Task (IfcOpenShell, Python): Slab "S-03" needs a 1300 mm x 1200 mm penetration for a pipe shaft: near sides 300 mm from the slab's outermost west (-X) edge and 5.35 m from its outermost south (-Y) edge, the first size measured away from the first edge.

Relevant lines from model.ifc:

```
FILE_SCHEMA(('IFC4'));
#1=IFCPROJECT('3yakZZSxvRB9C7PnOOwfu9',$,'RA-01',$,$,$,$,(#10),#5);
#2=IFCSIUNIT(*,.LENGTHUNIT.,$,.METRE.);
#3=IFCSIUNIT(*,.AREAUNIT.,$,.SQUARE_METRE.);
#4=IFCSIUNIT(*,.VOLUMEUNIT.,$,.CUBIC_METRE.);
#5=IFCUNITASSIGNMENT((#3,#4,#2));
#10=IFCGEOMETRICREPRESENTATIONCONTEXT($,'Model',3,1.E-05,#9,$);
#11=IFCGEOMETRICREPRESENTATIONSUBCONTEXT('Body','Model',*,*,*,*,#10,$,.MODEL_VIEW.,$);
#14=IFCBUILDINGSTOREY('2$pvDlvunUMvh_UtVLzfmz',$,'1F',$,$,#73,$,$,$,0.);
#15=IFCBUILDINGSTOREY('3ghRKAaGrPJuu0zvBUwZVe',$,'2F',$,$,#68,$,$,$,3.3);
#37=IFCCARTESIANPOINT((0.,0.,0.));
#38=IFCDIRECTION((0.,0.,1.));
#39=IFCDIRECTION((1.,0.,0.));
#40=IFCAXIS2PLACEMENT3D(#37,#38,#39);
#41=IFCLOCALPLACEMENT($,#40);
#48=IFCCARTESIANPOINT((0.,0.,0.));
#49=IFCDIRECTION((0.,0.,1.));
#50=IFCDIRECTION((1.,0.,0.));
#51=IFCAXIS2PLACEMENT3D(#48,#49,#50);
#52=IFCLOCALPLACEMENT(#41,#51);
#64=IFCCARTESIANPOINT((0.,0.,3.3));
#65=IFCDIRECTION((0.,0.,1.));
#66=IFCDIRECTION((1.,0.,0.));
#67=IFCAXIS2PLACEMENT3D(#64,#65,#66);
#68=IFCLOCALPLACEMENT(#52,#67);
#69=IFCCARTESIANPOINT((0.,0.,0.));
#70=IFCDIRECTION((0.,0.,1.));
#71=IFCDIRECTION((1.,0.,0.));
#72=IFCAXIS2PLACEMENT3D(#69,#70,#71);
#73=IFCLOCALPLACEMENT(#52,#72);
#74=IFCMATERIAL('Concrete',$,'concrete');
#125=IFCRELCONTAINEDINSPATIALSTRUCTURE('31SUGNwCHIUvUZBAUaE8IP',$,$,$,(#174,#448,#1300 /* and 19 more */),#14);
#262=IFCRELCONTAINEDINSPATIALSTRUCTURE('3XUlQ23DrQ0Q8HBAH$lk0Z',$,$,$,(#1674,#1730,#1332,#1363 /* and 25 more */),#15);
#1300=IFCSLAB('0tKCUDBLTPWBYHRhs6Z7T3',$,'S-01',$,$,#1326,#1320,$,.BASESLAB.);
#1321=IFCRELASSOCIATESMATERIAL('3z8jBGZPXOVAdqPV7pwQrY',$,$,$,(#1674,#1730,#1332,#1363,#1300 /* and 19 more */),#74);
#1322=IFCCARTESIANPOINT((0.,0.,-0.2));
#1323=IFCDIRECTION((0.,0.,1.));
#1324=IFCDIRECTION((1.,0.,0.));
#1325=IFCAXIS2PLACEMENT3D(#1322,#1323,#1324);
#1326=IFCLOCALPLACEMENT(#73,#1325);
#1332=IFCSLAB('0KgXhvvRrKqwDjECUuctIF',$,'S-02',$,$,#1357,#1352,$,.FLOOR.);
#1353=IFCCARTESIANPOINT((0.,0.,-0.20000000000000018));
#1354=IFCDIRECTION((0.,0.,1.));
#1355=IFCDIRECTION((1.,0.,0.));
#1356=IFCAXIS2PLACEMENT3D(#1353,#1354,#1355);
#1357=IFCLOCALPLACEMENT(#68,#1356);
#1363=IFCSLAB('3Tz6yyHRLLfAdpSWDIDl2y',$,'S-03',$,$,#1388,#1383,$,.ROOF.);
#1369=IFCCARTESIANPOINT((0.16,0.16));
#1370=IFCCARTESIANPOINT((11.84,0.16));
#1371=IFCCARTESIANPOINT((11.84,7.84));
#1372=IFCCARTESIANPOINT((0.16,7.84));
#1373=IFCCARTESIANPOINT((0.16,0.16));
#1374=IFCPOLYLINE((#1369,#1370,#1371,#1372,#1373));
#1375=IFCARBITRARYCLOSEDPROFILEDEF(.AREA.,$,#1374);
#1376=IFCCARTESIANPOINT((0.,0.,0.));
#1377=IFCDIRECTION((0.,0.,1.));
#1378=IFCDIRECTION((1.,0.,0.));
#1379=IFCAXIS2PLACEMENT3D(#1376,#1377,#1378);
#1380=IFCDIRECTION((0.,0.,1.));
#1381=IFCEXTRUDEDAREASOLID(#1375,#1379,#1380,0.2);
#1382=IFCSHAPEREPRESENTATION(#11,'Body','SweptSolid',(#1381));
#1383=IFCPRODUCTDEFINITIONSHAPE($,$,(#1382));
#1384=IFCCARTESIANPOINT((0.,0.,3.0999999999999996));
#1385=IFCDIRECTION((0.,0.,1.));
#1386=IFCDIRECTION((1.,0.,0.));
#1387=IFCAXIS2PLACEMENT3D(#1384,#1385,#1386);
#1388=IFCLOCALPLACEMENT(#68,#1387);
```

```python
import numpy as np
import ifcopenshell
import ifcopenshell.api.feature
import ifcopenshell.api.geometry
import ifcopenshell.api.root
import ifcopenshell.geom
import ifcopenshell.util.placement
import ifcopenshell.util.representation
import ifcopenshell.util.shape
import ifcopenshell.util.unit

model = ifcopenshell.open("model.ifc")
unit_scale = ifcopenshell.util.unit.calculate_unit_scale(model)
settings = ifcopenshell.geom.settings()


def volume(element):
    """Net volume in cubic metres, openings subtracted."""
    shape = ifcopenshell.geom.create_shape(settings, element)
    return ifcopenshell.util.shape.get_volume(shape.geometry)


slab = model.by_id(1363)
before = volume(slab)

# Extent in the slab's own axes, in metres. The edges named are its -X and -Y sides.
slab_shape = ifcopenshell.geom.create_shape(settings, slab)
vertices = ifcopenshell.util.shape.get_vertices(slab_shape.geometry)
x_min, y_min, bottom = vertices.min(axis=0)
top = vertices[:, 2].max()

opening = ifcopenshell.api.root.create_entity(model, ifc_class="IfcOpeningElement", name="Pipe shaft opening", predefined_type="OPENING")
context = ifcopenshell.util.representation.get_context(model, "Model", "Body", "MODEL_VIEW")
width, depth = 1.3, 1.2
outline = [(0.0, 0.0), (width, 0.0), (width, depth), (0.0, depth), (0.0, 0.0)]
# Overshoot both faces by 50 mm so the cut is clean.
shape = ifcopenshell.api.geometry.add_slab_representation(
    model, context=context, depth=top - bottom + 0.1, polyline=outline
)
ifcopenshell.api.geometry.assign_representation(model, product=opening, representation=shape)

matrix = ifcopenshell.util.placement.get_local_placement(slab.ObjectPlacement)
matrix[:, 3] = matrix @ np.append(np.array([x_min + 0.3, y_min + 5.35, bottom - 0.05]) / unit_scale, 1.0)
ifcopenshell.api.geometry.edit_object_placement(model, product=opening, matrix=matrix, is_si=False)
ifcopenshell.api.feature.add_feature(model, feature=opening, element=slab)

after = volume(slab)

print(f"slab volume {before:.3f} -> {after:.3f} m3")

model.write("model-out.ifc")
```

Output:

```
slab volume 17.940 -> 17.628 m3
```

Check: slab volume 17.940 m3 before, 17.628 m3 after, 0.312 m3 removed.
